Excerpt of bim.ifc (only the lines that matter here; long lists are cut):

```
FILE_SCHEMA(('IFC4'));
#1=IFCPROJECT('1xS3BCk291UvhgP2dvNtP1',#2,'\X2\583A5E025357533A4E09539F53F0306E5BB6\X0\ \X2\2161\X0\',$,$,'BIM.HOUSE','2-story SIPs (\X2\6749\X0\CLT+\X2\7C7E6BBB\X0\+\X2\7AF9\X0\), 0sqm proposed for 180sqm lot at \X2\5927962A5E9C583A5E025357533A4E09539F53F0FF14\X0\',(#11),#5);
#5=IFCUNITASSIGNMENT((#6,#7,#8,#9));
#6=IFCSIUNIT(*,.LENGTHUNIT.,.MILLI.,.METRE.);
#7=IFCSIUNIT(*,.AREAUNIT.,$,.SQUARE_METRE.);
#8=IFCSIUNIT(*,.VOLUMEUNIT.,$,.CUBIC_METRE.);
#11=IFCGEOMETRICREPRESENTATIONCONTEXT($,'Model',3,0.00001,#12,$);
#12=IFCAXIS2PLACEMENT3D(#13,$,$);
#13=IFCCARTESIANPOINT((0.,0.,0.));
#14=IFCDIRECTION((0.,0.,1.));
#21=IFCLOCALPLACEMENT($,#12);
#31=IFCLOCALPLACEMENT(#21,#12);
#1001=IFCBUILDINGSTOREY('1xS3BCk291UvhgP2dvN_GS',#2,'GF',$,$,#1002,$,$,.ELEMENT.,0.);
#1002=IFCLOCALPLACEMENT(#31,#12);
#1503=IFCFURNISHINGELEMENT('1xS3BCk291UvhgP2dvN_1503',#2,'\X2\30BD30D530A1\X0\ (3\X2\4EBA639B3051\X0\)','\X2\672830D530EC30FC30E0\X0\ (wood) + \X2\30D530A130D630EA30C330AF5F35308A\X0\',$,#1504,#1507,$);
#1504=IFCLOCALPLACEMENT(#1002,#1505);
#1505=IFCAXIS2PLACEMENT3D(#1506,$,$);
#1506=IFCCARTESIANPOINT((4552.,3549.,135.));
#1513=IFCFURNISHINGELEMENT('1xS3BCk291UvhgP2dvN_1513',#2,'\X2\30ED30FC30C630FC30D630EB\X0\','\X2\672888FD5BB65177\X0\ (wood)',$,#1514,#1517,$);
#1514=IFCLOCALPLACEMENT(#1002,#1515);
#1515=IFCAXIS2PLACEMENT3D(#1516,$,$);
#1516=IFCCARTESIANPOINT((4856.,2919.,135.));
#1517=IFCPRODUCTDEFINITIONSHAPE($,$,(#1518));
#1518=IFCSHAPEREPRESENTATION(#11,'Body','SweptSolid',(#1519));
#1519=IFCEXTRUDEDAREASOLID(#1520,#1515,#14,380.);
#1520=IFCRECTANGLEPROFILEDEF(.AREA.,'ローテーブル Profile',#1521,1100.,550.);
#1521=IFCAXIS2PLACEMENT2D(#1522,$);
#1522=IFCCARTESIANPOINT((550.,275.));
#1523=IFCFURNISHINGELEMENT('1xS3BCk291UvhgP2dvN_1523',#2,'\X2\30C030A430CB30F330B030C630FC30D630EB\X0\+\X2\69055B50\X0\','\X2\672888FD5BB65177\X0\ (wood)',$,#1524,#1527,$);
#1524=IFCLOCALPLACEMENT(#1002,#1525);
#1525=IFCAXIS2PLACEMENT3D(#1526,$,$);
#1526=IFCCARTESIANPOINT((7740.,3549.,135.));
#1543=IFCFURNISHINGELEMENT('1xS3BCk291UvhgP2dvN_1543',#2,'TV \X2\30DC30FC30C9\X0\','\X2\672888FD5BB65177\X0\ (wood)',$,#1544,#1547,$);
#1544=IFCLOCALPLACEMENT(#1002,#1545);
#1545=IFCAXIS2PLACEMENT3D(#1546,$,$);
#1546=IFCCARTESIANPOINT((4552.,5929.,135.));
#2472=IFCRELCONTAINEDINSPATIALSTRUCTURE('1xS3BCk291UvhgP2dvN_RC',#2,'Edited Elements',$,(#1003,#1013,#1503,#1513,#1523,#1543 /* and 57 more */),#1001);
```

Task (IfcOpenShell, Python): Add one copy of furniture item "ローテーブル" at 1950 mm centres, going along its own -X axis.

```python
import ifcopenshell
import ifcopenshell.api.geometry
import ifcopenshell.api.root
import ifcopenshell.util.element
import ifcopenshell.util.placement

model = ifcopenshell.open("bim.ifc")


def reuse_history(source, copy):
    """copy_class also copies each property set's owner history, people and application; keep the originals."""
    for rel in copy.IsDefinedBy:
        if rel.is_a("IfcRelDefinesByProperties") and (history := rel.RelatingPropertyDefinition.OwnerHistory):
            rel.RelatingPropertyDefinition.OwnerHistory = source.OwnerHistory
            ifcopenshell.util.element.remove_deep2(model, history)


source = model.by_id(1513)
base = ifcopenshell.util.placement.get_local_placement(source.ObjectPlacement)
step = -base[:3, 0] * 1950.0

for i in range(1, 2):
    copy = ifcopenshell.api.root.copy_class(model, product=source)
    copy.Representation = ifcopenshell.util.element.copy_deep(
        model, source.Representation, exclude=["IfcGeometricRepresentationContext", "IfcRepresentationMap"]
    )
    reuse_history(source, copy)
    matrix = base.copy()
    matrix[:3, 3] += i * step
    print("added at", matrix[:3, 3].round(3) + 0.0)
    ifcopenshell.api.geometry.edit_object_placement(model, product=copy, matrix=matrix, is_si=False)

model.write("bim_updated.ifc")
```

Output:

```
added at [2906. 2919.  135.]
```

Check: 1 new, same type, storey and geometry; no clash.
